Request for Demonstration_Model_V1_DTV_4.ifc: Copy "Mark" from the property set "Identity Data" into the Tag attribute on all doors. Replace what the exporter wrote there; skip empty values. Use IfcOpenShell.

First a look at what the model holds.

```python
import ifcopenshell
import ifcopenshell.util.element

model = ifcopenshell.open("Demonstration_Model_V1_DTV_4.ifc")
print(model.schema)
doors = model.by_type("IfcDoor")
print(len(doors), "doors")
for e in doors[:8]:
    source = ifcopenshell.util.element.get_pset(e, "Identity Data", "Mark")
    target = e.Tag
    print(e.id(), repr(source), repr(target), sep=" | ")
```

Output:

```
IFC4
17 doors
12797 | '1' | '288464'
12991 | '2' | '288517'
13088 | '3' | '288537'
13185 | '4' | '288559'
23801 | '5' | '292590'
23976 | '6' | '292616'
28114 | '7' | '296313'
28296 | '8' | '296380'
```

```python
import ifcopenshell
import ifcopenshell.util.element

model = ifcopenshell.open("Demonstration_Model_V1_DTV_4.ifc")

count = 0
for e in model.by_type("IfcDoor"):
    value = ifcopenshell.util.element.get_pset(e, "Identity Data", "Mark")
    current = e.Tag
    if not value or not value.strip() or current == value:
        continue
    e.Tag = value
    count += 1

print(count, "doors updated")

model.write("Demonstration_Model_V1_DTV_4-out.ifc")
```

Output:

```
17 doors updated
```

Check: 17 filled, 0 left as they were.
